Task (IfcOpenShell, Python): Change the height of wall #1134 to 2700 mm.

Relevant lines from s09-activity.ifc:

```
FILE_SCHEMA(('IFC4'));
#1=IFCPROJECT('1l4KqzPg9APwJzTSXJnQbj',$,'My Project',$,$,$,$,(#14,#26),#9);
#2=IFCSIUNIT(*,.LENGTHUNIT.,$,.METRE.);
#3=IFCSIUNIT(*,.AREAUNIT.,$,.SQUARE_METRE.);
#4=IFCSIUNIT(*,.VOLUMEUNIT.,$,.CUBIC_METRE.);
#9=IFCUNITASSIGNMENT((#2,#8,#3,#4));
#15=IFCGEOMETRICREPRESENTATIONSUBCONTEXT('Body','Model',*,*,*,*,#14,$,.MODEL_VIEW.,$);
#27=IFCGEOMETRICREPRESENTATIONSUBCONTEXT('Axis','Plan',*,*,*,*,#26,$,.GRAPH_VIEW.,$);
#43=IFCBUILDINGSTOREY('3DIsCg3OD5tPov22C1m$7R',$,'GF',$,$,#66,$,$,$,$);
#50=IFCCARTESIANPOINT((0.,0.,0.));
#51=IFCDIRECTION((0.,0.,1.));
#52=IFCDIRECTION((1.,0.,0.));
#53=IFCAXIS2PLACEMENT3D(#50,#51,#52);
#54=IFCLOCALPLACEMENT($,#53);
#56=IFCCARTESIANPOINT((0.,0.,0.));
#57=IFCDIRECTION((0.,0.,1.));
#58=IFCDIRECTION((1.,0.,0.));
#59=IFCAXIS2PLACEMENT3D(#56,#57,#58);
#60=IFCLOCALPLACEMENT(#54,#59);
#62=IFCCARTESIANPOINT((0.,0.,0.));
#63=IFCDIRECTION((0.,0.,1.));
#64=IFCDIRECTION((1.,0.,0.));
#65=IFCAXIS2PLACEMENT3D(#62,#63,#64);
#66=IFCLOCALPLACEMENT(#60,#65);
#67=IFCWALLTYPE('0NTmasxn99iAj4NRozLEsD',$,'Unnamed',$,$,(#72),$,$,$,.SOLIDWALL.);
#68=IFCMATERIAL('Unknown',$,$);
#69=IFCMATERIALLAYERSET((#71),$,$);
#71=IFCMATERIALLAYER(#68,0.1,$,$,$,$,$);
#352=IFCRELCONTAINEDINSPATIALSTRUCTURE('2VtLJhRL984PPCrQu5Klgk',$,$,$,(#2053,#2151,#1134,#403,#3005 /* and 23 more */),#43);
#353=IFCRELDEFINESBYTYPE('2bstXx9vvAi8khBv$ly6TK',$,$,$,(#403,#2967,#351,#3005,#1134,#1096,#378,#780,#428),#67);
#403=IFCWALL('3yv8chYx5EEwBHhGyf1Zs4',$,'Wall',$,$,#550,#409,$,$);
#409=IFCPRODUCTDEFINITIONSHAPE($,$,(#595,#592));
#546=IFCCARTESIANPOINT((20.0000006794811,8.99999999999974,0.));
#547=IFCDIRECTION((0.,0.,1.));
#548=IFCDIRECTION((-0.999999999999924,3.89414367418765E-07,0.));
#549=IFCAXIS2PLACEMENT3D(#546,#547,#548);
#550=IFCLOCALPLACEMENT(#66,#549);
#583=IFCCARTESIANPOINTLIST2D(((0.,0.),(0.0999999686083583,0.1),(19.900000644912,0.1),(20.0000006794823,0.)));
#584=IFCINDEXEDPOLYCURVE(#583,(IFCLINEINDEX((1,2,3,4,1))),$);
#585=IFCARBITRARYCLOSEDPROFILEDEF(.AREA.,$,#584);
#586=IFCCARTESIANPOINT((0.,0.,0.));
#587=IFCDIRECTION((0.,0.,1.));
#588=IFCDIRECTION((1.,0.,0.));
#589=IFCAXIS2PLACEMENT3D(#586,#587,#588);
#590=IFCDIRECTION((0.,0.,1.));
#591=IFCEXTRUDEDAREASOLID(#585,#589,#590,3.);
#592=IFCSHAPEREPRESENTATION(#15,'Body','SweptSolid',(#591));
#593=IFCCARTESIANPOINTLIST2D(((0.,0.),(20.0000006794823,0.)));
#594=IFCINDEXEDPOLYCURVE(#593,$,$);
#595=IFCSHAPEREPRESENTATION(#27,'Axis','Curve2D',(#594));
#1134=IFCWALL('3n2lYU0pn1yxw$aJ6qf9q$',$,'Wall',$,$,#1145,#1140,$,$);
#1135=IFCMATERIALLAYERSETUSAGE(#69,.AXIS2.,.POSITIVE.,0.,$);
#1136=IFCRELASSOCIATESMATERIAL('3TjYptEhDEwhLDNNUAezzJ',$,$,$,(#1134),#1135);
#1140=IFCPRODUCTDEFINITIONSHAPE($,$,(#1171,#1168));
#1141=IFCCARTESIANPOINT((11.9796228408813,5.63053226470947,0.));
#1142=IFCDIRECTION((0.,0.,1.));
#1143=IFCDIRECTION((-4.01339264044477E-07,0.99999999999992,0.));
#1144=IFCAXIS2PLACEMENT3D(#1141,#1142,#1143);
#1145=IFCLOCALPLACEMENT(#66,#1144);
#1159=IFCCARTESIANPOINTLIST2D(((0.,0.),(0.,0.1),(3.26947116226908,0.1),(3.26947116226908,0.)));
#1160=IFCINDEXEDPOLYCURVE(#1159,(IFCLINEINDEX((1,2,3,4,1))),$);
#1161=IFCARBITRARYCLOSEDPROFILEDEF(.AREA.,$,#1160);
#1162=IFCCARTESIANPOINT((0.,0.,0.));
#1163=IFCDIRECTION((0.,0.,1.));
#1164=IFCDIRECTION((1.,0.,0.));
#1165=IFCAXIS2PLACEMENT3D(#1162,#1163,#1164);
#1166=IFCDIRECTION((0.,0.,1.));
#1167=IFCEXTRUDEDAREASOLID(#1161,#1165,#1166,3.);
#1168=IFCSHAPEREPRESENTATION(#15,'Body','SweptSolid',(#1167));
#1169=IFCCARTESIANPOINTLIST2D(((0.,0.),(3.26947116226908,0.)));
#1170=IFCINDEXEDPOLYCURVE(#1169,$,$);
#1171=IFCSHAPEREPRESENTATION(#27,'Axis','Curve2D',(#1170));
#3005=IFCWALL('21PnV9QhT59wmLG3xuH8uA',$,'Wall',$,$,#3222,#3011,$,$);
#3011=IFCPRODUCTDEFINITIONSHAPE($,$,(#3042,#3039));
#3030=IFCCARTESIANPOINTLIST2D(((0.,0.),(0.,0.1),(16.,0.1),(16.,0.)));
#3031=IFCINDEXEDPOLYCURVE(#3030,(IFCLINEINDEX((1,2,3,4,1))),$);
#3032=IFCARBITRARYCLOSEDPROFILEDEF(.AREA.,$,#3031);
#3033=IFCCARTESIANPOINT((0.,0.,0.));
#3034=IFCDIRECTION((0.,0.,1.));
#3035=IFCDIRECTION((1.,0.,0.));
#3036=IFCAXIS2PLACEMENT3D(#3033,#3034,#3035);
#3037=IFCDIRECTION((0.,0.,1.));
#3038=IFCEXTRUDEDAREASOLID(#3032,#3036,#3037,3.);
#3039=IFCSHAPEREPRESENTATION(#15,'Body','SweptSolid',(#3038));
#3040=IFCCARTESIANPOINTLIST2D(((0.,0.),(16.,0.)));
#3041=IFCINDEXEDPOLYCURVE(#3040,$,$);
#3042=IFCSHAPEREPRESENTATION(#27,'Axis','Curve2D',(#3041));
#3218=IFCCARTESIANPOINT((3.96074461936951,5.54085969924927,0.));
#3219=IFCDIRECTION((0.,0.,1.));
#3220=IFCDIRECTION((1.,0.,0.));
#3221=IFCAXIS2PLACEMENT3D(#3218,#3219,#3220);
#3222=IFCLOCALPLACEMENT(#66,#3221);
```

```python
import ifcopenshell
import ifcopenshell.geom
import ifcopenshell.util.representation
import ifcopenshell.util.shape

model = ifcopenshell.open("s09-activity.ifc")
settings = ifcopenshell.geom.settings()


def volume(element):
    """Net volume in cubic metres, openings subtracted."""
    shape = ifcopenshell.geom.create_shape(settings, element)
    return ifcopenshell.util.shape.get_volume(shape.geometry)


wall = model.by_guid("3n2lYU0pn1yxw$aJ6qf9q$")
before = volume(wall)

body = ifcopenshell.util.representation.get_representation(wall, "Model", "Body")
solid = body.Items[0]
old_height = solid.Depth
solid.Depth = 2.7
after = volume(wall)

print(f"height {old_height:g} -> {solid.Depth:g}, volume {before:.3f} -> {after:.3f} m3")

model.write("s09-activity-out.ifc")
```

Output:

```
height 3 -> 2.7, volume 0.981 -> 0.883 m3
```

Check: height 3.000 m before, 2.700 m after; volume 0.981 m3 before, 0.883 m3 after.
